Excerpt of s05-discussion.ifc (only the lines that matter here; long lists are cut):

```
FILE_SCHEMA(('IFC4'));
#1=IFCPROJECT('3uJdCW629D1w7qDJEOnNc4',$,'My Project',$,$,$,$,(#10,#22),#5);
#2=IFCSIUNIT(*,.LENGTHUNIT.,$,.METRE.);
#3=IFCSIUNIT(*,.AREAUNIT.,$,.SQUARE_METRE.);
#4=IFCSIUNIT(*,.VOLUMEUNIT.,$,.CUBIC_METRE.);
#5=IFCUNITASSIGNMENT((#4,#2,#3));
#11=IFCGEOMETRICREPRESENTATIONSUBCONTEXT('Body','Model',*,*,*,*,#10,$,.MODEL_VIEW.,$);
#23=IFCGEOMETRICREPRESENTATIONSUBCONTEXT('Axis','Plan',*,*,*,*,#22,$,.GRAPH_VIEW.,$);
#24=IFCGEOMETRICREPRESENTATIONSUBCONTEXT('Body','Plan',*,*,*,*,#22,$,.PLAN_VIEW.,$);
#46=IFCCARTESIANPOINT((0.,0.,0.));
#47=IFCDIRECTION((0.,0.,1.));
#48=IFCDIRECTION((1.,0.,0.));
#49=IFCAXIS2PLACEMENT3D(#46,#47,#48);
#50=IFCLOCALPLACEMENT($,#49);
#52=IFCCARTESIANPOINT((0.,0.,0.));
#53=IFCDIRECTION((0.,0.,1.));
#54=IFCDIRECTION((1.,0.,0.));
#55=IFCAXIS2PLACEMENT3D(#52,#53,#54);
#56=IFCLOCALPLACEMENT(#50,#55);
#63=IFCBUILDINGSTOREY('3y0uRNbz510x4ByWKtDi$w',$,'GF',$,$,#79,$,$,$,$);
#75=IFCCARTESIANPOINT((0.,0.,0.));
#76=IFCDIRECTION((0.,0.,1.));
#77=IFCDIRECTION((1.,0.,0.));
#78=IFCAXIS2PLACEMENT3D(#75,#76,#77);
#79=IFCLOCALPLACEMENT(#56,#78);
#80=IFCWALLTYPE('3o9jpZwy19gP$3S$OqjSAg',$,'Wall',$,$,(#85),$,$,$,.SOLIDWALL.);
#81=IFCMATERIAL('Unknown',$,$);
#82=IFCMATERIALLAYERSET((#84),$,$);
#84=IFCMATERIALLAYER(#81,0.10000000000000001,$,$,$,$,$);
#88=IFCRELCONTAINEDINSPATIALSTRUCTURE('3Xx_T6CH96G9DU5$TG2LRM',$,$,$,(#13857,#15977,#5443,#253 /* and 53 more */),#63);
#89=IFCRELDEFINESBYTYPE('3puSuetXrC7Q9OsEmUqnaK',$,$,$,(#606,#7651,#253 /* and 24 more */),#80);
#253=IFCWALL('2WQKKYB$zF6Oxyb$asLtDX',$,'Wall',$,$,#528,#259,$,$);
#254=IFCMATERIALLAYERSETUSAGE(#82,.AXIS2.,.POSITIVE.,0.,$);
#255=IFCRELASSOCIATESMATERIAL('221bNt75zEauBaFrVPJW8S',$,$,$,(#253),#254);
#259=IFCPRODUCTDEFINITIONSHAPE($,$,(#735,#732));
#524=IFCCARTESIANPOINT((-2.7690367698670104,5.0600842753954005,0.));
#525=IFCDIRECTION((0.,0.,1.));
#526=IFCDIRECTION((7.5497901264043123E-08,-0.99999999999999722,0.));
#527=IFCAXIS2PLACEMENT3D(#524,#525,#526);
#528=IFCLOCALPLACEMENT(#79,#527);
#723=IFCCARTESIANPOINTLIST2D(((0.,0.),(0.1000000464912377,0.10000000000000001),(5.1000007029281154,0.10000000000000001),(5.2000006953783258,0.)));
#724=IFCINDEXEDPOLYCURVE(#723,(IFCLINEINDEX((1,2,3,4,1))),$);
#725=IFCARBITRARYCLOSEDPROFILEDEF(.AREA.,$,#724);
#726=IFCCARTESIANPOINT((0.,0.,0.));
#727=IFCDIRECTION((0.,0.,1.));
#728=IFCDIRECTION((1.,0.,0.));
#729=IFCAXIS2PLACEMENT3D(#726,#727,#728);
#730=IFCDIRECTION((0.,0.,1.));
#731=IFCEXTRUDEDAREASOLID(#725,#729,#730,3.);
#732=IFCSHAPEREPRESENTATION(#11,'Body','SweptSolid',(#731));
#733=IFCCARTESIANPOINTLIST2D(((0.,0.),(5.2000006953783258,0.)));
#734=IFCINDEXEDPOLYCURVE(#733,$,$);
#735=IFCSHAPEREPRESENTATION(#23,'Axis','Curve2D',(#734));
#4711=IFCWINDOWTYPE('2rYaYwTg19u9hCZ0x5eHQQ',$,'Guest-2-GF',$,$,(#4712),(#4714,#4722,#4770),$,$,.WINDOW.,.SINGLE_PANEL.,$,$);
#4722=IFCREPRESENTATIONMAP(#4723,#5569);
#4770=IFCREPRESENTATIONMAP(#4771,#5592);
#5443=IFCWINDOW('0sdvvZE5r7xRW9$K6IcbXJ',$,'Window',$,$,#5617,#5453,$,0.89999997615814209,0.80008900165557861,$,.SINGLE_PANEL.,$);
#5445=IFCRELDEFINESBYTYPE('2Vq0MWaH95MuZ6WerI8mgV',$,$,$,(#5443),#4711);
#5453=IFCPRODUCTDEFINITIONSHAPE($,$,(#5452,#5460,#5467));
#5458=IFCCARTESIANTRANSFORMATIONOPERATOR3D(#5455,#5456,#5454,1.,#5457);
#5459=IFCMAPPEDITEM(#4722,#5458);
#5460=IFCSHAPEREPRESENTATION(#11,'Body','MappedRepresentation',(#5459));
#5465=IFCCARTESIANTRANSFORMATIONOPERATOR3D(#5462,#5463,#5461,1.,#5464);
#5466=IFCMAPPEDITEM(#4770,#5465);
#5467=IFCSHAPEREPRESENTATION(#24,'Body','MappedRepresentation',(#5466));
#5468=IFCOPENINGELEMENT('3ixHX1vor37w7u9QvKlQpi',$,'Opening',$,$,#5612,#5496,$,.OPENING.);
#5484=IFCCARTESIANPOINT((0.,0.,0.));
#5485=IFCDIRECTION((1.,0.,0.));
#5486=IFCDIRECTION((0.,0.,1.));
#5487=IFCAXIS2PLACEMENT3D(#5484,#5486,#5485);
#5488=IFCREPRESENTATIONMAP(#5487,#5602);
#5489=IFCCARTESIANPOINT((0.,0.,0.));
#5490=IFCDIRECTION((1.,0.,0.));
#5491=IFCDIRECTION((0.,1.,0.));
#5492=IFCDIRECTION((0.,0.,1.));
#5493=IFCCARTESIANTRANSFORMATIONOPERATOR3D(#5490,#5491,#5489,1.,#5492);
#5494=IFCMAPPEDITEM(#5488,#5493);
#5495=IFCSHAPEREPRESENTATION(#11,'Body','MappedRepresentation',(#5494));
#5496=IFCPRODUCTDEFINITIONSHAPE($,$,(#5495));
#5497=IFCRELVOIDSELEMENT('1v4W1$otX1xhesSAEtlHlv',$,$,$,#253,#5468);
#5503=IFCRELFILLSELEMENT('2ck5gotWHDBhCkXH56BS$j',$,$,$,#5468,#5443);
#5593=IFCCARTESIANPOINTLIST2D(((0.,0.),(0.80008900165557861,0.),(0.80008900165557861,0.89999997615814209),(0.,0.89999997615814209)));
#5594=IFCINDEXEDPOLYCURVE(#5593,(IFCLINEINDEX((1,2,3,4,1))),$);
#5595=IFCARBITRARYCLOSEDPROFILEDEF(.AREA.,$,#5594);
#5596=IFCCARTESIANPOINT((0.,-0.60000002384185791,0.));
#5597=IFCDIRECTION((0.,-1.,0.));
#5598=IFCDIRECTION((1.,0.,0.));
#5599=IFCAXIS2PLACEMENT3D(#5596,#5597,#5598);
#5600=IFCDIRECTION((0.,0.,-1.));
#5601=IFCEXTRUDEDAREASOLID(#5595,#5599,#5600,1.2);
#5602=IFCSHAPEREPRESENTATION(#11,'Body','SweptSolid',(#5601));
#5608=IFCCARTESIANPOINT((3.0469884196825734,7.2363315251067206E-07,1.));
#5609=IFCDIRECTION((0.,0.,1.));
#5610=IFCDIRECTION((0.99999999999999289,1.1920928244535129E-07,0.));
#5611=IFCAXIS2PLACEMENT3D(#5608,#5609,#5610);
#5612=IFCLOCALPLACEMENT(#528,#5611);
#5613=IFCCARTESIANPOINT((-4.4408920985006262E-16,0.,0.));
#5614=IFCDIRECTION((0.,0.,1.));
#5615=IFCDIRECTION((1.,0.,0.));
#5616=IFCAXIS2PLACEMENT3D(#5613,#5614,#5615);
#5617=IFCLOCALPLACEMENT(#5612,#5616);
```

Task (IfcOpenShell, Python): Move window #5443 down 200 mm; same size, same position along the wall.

```python
import numpy as np
import ifcopenshell
import ifcopenshell.api.geometry
import ifcopenshell.util.placement
import ifcopenshell.util.unit

model = ifcopenshell.open("s05-discussion.ifc")
unit_scale = ifcopenshell.util.unit.calculate_unit_scale(model)

window = model.by_guid("0sdvvZE5r7xRW9$K6IcbXJ")
opening = window.FillsVoids[0].RelatingOpeningElement
dz = -0.2

shift = np.array([0.0, 0.0, dz])
# The window is placed relative to its opening, so it follows when the opening moves.
matrix = ifcopenshell.util.placement.get_local_placement(opening.ObjectPlacement)
matrix[:3, 3] += shift
ifcopenshell.api.geometry.edit_object_placement(
    model, product=opening, matrix=matrix, is_si=False, should_transform_children=True
)

print(f"moved by {dz * unit_scale:+.3f} m")

model.write("s05-discussion_rev.ifc")
```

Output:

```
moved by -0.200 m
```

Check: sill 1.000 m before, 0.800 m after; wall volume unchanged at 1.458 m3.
